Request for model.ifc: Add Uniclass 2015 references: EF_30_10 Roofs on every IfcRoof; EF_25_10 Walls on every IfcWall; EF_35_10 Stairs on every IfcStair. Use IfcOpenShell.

First a look at what the model holds.

```python
import ifcopenshell

model = ifcopenshell.open("model.ifc")
print(model.schema)
print("classifications:", [c.Name for c in model.by_type("IfcClassification")])
for ifc_class in ("IfcDoor", "IfcRoof", "IfcStair", "IfcWall", "IfcWindow"):
    print(ifc_class, len(model.by_type(ifc_class)))
```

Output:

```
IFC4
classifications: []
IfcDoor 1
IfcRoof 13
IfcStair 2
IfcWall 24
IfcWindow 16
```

```python
import ifcopenshell
import ifcopenshell.api.classification

model = ifcopenshell.open("model.ifc")

system = ifcopenshell.api.classification.add_classification(model, classification="Uniclass 2015")

codes = {
    "IfcRoof": ("EF_30_10", "Roofs"),
    "IfcWall": ("EF_25_10", "Walls"),
    "IfcStair": ("EF_35_10", "Stairs"),
}
for ifc_class, (code, name) in codes.items():
    products = model.by_type(ifc_class)
    ifcopenshell.api.classification.add_reference(
        model, products=products, classification=system, identification=code, name=name
    )
    print(code, len(products))

model.write("model-out.ifc")
```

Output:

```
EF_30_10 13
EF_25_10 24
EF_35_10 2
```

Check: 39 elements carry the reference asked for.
